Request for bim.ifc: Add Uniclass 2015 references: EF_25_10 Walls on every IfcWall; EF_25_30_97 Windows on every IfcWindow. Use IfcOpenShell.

First a look at what the model holds.

```python
import ifcopenshell

model = ifcopenshell.open("bim.ifc")
print(model.schema)
print("classifications:", [c.Name for c in model.by_type("IfcClassification")])
for ifc_class in ("IfcDoor", "IfcRoof", "IfcStair", "IfcWall", "IfcWindow"):
    print(ifc_class, len(model.by_type(ifc_class)))
```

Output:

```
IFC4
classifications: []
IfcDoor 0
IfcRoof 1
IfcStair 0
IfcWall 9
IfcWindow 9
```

```python
import ifcopenshell
import ifcopenshell.api.classification

model = ifcopenshell.open("bim.ifc")

system = ifcopenshell.api.classification.add_classification(model, classification="Uniclass 2015")

codes = {
    "IfcWall": ("EF_25_10", "Walls"),
    "IfcWindow": ("EF_25_30_97", "Windows"),
}
for ifc_class, (code, name) in codes.items():
    products = model.by_type(ifc_class)
    ifcopenshell.api.classification.add_reference(
        model, products=products, classification=system, identification=code, name=name
    )
    print(code, len(products))

model.write("bim_v2.ifc")
```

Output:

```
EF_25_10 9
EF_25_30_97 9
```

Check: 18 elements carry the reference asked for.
